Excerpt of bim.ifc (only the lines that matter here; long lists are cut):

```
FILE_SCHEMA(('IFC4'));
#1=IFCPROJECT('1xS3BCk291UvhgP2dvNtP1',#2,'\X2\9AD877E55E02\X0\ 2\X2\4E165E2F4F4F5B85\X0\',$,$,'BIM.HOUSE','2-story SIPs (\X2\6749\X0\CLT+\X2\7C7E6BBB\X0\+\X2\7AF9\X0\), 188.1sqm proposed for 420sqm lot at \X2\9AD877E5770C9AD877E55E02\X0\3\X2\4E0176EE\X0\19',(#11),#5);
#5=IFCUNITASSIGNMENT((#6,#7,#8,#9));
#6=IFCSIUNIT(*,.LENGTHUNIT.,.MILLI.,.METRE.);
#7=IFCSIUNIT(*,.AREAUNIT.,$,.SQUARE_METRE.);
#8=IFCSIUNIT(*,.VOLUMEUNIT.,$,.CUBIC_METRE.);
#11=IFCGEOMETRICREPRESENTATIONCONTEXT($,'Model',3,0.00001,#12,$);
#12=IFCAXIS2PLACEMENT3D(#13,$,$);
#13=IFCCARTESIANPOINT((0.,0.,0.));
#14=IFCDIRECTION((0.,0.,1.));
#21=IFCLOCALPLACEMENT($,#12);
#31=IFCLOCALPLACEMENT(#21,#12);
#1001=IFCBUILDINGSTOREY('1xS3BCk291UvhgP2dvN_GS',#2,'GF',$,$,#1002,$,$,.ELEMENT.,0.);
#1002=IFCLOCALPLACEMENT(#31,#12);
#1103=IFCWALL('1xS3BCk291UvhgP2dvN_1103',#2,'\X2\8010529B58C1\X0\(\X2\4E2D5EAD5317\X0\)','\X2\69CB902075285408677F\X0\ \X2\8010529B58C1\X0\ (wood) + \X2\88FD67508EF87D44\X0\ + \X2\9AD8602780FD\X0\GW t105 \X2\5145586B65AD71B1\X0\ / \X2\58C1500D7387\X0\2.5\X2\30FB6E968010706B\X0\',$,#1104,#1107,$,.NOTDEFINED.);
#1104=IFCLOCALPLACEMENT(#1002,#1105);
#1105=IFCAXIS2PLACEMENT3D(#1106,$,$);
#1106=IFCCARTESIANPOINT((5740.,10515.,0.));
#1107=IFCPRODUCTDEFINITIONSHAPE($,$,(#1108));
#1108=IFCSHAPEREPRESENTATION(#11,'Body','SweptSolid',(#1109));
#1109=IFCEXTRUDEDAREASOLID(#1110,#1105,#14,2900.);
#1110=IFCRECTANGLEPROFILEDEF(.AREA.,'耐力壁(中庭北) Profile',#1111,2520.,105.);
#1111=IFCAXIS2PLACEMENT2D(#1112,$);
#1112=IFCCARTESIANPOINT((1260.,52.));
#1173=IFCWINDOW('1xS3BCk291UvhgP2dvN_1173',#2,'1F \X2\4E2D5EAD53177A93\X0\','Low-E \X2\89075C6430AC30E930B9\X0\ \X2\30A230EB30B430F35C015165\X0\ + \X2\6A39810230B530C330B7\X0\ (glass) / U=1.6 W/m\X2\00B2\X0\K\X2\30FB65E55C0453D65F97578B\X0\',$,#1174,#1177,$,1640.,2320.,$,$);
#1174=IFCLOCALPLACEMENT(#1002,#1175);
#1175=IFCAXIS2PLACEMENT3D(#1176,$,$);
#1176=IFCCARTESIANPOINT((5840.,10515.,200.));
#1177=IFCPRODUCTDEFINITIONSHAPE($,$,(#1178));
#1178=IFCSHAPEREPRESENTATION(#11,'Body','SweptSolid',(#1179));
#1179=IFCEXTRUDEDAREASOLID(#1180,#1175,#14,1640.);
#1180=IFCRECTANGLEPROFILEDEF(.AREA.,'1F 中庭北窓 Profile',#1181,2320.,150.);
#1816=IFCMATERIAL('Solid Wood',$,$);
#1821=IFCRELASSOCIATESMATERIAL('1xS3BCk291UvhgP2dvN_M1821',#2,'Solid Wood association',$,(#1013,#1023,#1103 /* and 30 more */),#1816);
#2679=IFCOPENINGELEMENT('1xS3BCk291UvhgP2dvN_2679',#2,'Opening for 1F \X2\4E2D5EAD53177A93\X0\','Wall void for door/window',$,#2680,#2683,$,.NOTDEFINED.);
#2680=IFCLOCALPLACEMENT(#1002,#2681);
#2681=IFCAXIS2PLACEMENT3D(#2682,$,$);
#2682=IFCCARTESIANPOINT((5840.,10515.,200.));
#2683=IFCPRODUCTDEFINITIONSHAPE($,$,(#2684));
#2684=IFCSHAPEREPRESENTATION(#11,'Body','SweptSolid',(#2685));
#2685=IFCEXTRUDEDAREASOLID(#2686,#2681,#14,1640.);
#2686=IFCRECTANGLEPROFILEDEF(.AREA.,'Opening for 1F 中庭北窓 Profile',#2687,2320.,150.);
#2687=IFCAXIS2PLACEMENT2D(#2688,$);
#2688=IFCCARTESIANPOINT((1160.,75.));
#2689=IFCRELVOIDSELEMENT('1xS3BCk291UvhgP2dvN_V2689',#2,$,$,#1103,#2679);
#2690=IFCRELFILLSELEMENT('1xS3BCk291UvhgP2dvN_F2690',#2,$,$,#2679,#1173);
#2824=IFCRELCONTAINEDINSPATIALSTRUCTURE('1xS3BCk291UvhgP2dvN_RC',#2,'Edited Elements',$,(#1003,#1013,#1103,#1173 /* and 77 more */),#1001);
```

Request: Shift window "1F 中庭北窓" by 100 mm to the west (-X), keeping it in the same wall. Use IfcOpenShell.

```python
import ifcopenshell
import ifcopenshell.api.geometry
import ifcopenshell.util.placement
import ifcopenshell.util.unit

model = ifcopenshell.open("bim.ifc")
unit_scale = ifcopenshell.util.unit.calculate_unit_scale(model)

window = model.by_guid("1xS3BCk291UvhgP2dvN_1173")
opening = window.FillsVoids[0].RelatingOpeningElement
wall = opening.VoidsElements[0].RelatingBuildingElement

wall_matrix = ifcopenshell.util.placement.get_local_placement(wall.ObjectPlacement)
shift = wall_matrix[:3, 0] * -0.1 / unit_scale
before = ifcopenshell.util.placement.get_local_placement(window.ObjectPlacement)[:3, 3].copy()

# The window is not placed relative to its opening, so move both.
for product in (opening, window):
    matrix = ifcopenshell.util.placement.get_local_placement(product.ObjectPlacement)
    matrix[:3, 3] += shift
    ifcopenshell.api.geometry.edit_object_placement(model, product=product, matrix=matrix, is_si=False)

after = ifcopenshell.util.placement.get_local_placement(window.ObjectPlacement)[:3, 3]
print("window moved by", (after - before).round(3) + 0.0)

model.write("bim_v2.ifc")
```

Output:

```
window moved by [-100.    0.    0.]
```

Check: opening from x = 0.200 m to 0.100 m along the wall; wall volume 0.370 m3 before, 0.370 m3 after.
